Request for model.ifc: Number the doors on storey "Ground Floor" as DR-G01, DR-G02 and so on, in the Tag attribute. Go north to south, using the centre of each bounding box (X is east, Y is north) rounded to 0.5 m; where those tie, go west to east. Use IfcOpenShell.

First a look at what the model holds.

```python
import ifcopenshell
import ifcopenshell.util.element
import ifcopenshell.util.placement

model = ifcopenshell.open("model.ifc")
print(model.schema)
storey = next(s for s in model.by_type("IfcBuildingStorey") if s.Name == "Ground Floor")
doors = [e for e in ifcopenshell.util.element.get_decomposition(storey) if e.is_a("IfcDoor")]
for e in sorted(doors, key=lambda e: e.id()):
    origin = ifcopenshell.util.placement.get_local_placement(e.ObjectPlacement)[:3, 3]
    print(e.id(), e.Tag, e.Name, origin.round(2) + 0.0, sep=" | ")
```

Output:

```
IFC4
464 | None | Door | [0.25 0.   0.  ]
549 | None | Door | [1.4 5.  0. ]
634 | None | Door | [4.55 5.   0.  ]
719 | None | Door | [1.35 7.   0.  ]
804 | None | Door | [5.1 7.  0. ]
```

```python
import ifcopenshell
import ifcopenshell.geom
import ifcopenshell.util.element
import ifcopenshell.util.shape

model = ifcopenshell.open("model.ifc")
settings = ifcopenshell.geom.settings()
settings.set("use-world-coords", True)


def centre(element):
    shape = ifcopenshell.geom.create_shape(settings, element)
    return ifcopenshell.util.shape.get_bbox_centroid(shape.geometry)


storey = next(s for s in model.by_type("IfcBuildingStorey") if s.Name == "Ground Floor")
doors = [e for e in ifcopenshell.util.element.get_decomposition(storey) if e.is_a("IfcDoor")]

# Insertion points can sit at a corner or the storey origin, so sort by the geometry (in metres).
centres = {e: centre(e) for e in doors}
doors.sort(key=lambda e: (-round(centres[e][1] / 0.5), centres[e][0]))

for i, e in enumerate(doors, start=1):
    number = f"DR-G{i:02d}"
    e.Tag = number
    print(e.id(), number)

model.write("model_rev.ifc")
```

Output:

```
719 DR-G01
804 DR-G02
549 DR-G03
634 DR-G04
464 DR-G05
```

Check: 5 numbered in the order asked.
